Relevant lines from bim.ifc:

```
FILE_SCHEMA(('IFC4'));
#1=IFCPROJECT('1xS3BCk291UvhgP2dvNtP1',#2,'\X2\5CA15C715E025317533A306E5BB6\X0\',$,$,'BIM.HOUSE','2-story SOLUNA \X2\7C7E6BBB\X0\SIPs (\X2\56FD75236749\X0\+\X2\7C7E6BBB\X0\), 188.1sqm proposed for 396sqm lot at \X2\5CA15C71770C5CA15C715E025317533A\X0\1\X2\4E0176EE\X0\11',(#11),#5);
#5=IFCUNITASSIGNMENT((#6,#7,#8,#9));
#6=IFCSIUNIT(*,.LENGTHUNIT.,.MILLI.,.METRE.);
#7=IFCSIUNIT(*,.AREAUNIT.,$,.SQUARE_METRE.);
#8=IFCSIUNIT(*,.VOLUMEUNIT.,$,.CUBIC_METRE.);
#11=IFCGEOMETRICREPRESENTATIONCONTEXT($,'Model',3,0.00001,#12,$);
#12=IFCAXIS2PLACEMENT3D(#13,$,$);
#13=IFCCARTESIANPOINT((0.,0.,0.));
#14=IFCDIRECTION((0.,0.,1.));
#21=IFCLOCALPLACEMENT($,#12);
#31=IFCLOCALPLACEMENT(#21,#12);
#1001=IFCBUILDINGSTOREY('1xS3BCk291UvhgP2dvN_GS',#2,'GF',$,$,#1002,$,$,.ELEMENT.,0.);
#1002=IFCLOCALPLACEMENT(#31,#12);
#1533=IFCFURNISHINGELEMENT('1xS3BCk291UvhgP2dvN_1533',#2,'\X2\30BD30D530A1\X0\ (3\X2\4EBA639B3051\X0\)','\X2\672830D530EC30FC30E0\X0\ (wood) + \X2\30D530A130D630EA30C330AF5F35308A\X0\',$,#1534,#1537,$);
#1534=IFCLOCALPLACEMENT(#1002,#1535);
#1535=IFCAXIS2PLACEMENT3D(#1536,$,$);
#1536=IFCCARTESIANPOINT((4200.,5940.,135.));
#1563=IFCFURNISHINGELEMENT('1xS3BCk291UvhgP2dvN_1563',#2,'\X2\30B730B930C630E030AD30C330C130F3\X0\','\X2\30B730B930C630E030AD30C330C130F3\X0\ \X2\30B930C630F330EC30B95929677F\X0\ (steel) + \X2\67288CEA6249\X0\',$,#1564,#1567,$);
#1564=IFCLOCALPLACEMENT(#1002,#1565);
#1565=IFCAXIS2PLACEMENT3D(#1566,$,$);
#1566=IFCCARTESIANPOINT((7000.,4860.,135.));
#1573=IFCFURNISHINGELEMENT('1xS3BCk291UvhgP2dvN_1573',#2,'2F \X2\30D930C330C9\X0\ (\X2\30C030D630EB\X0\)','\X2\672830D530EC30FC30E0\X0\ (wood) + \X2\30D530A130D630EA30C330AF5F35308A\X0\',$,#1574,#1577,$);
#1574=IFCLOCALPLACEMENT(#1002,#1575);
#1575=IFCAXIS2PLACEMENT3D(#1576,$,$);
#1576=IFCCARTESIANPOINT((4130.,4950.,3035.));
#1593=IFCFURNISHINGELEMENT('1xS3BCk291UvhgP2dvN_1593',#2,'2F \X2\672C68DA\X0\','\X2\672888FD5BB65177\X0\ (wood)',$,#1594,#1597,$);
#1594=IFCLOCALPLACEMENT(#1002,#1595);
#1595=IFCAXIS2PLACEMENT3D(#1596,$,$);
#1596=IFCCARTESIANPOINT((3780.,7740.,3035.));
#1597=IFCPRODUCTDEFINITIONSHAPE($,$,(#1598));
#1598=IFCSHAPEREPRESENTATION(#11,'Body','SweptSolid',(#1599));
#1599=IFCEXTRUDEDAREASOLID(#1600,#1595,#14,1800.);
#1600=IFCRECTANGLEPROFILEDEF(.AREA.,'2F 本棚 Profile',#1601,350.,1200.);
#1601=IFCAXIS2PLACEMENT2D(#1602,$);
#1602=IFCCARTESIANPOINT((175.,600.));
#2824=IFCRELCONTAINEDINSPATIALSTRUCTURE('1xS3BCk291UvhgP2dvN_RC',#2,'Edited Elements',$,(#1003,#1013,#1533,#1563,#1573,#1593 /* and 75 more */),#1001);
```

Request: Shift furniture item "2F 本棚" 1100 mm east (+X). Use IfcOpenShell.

```python
import ifcopenshell
import ifcopenshell.api.geometry
import ifcopenshell.util.placement

model = ifcopenshell.open("bim.ifc")

item = model.by_id(1593)
matrix = ifcopenshell.util.placement.get_local_placement(item.ObjectPlacement)
matrix[0, 3] += 1100.0
ifcopenshell.api.geometry.edit_object_placement(model, product=item, matrix=matrix, is_si=False)

print(ifcopenshell.util.placement.get_local_placement(item.ObjectPlacement).round(3) + 0.0)

model.write("bim_edited.ifc")
```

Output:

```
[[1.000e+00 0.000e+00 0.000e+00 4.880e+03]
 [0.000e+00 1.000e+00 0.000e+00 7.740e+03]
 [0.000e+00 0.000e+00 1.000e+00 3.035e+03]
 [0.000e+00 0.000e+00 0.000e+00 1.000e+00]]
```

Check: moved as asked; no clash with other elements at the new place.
